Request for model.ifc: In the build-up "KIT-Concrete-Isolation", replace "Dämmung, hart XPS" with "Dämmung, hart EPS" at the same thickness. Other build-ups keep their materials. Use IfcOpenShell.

First a look at what the model holds.

```python
import ifcopenshell
import ifcopenshell.util.element

model = ifcopenshell.open("model.ifc")
print(model.schema)
for layer_set in model.by_type("IfcMaterialLayerSet"):
    if layer_set.LayerSetName == "KIT-Concrete-Isolation":
        for layer in layer_set.MaterialLayers:
            print(layer.id(), layer.Material and layer.Material.Name, layer.LayerThickness, sep=" | ")
        print(len(ifcopenshell.util.element.get_elements_by_material(model, layer_set)), "elements and types use it")
print(sorted(m.Name for m in model.by_type("IfcMaterial") if m.Name)[:60])
```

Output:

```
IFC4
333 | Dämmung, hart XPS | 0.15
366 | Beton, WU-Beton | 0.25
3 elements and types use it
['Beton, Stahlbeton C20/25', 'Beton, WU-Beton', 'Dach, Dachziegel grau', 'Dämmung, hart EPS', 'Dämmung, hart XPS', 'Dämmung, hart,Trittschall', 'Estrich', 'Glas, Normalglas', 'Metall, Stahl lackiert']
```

```python
import ifcopenshell
import ifcopenshell.api.material

model = ifcopenshell.open("model.ifc")

layer_set = next(s for s in model.by_type("IfcMaterialLayerSet") if s.LayerSetName == "KIT-Concrete-Isolation")
layer = next(l for l in layer_set.MaterialLayers if l.Material and l.Material.Name == "Dämmung, hart XPS")
material = next(m for m in model.by_type("IfcMaterial") if m.Name == "Dämmung, hart EPS")

# Point this one layer at the other material; renaming the old one would change it everywhere.
ifcopenshell.api.material.edit_layer(model, layer=layer, attributes={}, material=material)

print([l.Material.Name if l.Material else None for l in layer_set.MaterialLayers])

model.write("model-out.ifc")
```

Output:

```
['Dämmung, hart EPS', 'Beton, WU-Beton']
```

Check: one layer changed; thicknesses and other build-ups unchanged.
